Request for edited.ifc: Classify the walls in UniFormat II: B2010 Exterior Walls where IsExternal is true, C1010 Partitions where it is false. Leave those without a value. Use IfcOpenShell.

First a look at what the model holds.

```python
import ifcopenshell
import ifcopenshell.util.element

model = ifcopenshell.open("edited.ifc")
print(model.schema)
print("classifications:", [c.Name for c in model.by_type("IfcClassification")])
values = [ifcopenshell.util.element.get_pset(e, "Pset_WallCommon", "IsExternal") for e in model.by_type("IfcWall")]
for value in (True, False, None):
    print("IsExternal", value, values.count(value))
```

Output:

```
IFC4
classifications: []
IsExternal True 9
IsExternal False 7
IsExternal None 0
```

```python
import ifcopenshell
import ifcopenshell.api.classification
import ifcopenshell.util.element

model = ifcopenshell.open("edited.ifc")

system = ifcopenshell.api.classification.add_classification(model, classification="UniFormat II")

walls = model.by_type("IfcWall")
external = {e: ifcopenshell.util.element.get_pset(e, "Pset_WallCommon", "IsExternal") for e in walls}
for flag, code, name in ((True, "B2010", "Exterior Walls"), (False, "C1010", "Partitions")):
    products = [e for e in walls if external[e] is flag]
    ifcopenshell.api.classification.add_reference(
        model, products=products, classification=system, identification=code, name=name
    )
    print(code, len(products))

model.write("edited_rev.ifc")
```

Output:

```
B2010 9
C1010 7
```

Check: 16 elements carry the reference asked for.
